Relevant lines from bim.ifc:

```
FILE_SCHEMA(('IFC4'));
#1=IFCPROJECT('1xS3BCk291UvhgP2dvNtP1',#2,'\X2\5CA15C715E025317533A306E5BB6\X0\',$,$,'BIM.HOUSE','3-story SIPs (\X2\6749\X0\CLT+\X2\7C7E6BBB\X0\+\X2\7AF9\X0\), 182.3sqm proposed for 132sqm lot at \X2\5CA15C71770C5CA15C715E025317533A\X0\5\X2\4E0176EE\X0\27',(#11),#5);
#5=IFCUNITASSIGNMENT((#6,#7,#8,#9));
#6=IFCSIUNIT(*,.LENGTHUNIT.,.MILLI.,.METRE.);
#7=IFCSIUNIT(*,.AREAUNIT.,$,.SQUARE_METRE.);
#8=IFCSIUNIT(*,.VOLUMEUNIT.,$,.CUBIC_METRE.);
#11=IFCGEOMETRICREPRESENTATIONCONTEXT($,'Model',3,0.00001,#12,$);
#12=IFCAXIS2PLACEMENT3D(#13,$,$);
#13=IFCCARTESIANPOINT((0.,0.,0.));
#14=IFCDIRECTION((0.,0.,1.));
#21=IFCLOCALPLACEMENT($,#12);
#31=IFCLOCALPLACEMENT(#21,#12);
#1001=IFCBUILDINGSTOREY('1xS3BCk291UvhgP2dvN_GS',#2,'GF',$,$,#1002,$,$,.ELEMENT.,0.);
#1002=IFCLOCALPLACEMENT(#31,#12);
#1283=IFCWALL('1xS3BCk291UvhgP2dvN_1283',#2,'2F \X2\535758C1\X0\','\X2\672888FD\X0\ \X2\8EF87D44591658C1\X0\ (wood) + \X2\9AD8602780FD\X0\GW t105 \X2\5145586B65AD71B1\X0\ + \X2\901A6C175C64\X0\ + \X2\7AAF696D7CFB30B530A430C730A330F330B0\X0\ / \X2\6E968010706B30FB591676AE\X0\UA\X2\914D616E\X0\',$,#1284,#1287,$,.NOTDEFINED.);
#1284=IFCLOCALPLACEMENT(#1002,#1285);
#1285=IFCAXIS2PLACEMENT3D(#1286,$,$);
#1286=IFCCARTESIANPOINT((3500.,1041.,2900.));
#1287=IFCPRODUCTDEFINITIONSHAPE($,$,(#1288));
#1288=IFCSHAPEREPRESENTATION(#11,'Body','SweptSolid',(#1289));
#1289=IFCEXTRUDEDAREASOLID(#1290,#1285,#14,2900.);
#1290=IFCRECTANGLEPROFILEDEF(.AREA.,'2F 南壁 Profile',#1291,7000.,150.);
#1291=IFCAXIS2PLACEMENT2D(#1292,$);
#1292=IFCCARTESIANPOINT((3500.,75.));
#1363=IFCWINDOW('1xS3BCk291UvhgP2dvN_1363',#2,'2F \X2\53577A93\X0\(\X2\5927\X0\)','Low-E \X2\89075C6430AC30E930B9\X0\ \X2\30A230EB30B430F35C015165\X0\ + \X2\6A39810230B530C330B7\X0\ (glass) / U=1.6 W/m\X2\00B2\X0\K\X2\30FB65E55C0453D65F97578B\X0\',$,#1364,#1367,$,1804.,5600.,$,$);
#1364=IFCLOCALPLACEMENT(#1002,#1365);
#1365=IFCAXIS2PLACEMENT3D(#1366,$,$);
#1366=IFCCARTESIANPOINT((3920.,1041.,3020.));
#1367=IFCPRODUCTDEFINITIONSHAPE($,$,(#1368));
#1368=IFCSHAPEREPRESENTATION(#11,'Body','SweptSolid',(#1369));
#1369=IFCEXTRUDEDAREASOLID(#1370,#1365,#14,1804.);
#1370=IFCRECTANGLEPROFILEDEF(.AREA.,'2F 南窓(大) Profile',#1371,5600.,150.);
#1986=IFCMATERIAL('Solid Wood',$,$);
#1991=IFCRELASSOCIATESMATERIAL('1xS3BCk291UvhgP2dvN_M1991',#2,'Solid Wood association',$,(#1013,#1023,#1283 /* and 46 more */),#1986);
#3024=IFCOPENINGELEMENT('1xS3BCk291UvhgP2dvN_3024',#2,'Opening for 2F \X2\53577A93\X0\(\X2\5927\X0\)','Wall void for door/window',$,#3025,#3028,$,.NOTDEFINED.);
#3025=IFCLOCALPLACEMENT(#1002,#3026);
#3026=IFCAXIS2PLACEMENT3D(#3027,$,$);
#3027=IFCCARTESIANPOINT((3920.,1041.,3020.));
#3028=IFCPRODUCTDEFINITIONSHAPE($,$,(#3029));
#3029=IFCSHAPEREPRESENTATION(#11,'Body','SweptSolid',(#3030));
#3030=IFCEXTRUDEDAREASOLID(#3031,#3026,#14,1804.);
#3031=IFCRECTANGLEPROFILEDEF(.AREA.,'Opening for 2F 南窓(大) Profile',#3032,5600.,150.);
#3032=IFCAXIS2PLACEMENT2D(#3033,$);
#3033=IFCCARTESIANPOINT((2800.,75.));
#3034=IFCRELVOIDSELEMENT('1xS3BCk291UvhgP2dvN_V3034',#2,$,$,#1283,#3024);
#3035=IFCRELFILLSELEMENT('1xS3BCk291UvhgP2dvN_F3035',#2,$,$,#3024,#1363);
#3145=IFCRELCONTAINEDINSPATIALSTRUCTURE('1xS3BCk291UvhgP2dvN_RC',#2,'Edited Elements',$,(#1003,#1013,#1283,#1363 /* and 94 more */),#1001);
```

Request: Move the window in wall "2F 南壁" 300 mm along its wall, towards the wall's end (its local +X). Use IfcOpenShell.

```python
import ifcopenshell
import ifcopenshell.api.geometry
import ifcopenshell.util.placement
import ifcopenshell.util.unit

model = ifcopenshell.open("bim.ifc")
unit_scale = ifcopenshell.util.unit.calculate_unit_scale(model)

window = model.by_guid("1xS3BCk291UvhgP2dvN_1363")
opening = window.FillsVoids[0].RelatingOpeningElement
wall = opening.VoidsElements[0].RelatingBuildingElement

wall_matrix = ifcopenshell.util.placement.get_local_placement(wall.ObjectPlacement)
shift = wall_matrix[:3, 0] * 0.3 / unit_scale
before = ifcopenshell.util.placement.get_local_placement(window.ObjectPlacement)[:3, 3].copy()

# The window is not placed relative to its opening, so move both.
for product in (opening, window):
    matrix = ifcopenshell.util.placement.get_local_placement(product.ObjectPlacement)
    matrix[:3, 3] += shift
    ifcopenshell.api.geometry.edit_object_placement(model, product=product, matrix=matrix, is_si=False)

after = ifcopenshell.util.placement.get_local_placement(window.ObjectPlacement)[:3, 3]
print("window moved by", (after - before).round(3) + 0.0)

model.write("bim_edited.ifc")
```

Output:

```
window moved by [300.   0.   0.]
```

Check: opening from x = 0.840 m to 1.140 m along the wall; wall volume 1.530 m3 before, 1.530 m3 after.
